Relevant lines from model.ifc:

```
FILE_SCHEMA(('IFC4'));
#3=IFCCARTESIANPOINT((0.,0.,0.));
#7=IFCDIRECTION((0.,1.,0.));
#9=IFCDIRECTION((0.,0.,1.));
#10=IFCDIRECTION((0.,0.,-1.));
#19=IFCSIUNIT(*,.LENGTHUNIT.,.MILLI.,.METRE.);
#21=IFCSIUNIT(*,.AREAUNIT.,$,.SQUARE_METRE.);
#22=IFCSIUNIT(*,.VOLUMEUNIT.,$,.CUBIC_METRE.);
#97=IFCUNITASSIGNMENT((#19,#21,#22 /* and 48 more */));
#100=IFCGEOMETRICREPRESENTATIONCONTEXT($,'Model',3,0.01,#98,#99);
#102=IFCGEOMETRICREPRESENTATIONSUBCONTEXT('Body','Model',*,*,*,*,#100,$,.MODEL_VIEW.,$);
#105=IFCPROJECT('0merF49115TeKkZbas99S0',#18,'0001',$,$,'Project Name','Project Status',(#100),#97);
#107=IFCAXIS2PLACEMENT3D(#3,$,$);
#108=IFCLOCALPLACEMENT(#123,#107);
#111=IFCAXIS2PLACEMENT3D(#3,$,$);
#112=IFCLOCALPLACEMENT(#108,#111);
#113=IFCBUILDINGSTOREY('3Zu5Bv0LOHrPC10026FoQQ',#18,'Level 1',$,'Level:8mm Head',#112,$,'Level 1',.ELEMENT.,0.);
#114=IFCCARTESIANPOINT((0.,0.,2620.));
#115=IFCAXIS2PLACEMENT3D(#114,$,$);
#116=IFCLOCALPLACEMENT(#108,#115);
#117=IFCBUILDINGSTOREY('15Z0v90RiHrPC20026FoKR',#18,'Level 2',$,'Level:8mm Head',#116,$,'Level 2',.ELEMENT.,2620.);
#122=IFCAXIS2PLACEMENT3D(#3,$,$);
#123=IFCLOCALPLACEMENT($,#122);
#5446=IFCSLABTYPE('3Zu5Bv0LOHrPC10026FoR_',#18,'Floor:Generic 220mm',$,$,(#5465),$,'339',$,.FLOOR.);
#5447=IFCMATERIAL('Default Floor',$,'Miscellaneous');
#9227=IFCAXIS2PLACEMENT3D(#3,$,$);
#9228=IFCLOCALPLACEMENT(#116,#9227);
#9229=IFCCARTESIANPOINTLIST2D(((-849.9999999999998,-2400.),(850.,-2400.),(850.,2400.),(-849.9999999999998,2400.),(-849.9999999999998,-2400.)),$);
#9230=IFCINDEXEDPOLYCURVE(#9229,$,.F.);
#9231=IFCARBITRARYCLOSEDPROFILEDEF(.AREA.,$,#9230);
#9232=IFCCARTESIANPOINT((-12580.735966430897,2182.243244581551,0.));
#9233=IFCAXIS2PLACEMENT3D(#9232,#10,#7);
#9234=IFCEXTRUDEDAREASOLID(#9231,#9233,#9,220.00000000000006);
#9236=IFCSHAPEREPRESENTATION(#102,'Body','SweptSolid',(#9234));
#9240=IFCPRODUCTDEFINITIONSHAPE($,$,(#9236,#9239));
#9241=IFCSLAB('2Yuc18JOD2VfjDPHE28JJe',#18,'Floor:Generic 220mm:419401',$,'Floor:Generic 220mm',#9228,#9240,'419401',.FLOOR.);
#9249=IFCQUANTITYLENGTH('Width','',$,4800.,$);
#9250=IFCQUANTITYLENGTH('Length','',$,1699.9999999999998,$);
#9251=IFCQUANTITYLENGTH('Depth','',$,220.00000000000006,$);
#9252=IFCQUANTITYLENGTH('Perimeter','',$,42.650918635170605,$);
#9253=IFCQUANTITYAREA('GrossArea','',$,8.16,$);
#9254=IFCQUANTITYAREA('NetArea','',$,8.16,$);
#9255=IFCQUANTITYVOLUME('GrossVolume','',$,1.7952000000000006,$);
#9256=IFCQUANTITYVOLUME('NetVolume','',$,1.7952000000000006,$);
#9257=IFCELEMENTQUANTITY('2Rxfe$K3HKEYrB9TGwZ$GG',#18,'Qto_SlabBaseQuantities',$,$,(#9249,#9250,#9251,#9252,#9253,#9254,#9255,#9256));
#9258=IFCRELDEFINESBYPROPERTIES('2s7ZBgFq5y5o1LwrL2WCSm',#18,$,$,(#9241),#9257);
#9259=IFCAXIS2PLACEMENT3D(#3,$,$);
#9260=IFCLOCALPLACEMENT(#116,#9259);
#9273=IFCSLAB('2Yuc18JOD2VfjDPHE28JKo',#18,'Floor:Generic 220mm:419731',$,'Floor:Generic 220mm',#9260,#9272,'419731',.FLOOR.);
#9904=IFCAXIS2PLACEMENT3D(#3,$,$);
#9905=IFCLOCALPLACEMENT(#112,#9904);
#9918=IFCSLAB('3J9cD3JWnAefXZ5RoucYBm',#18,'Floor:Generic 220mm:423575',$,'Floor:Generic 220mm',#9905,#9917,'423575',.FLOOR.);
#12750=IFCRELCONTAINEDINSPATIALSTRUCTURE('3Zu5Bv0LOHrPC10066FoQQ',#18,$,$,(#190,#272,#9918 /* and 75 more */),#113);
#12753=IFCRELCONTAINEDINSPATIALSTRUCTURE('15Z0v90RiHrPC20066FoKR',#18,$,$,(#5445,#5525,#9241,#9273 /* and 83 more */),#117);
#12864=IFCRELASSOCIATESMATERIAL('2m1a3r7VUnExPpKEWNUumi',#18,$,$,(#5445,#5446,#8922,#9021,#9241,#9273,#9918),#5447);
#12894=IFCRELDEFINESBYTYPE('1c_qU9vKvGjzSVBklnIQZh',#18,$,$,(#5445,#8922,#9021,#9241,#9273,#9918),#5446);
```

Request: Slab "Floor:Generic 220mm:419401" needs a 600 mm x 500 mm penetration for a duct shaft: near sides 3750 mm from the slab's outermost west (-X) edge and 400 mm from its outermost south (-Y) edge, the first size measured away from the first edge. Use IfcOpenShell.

```python
import numpy as np
import ifcopenshell
import ifcopenshell.api.feature
import ifcopenshell.api.geometry
import ifcopenshell.api.pset
import ifcopenshell.api.root
import ifcopenshell.geom
import ifcopenshell.util.element
import ifcopenshell.util.placement
import ifcopenshell.util.representation
import ifcopenshell.util.shape
import ifcopenshell.util.unit

model = ifcopenshell.open("model.ifc")
unit_scale = ifcopenshell.util.unit.calculate_unit_scale(model)
area_scale = ifcopenshell.util.unit.calculate_unit_scale(model, "AREAUNIT")
volume_scale = ifcopenshell.util.unit.calculate_unit_scale(model, "VOLUMEUNIT")
settings = ifcopenshell.geom.settings()


def volume(element):
    """Net volume in cubic metres, openings subtracted."""
    shape = ifcopenshell.geom.create_shape(settings, element)
    return ifcopenshell.util.shape.get_volume(shape.geometry)


slab = model.by_guid("2Yuc18JOD2VfjDPHE28JJe")
before = volume(slab)

# Extent in the slab's own axes, in metres. The edges named are its -X and -Y sides.
slab_shape = ifcopenshell.geom.create_shape(settings, slab)
vertices = ifcopenshell.util.shape.get_vertices(slab_shape.geometry)
x_min, y_min, bottom = vertices.min(axis=0)
top = vertices[:, 2].max()

opening = ifcopenshell.api.root.create_entity(model, ifc_class="IfcOpeningElement", name="Duct shaft opening", predefined_type="OPENING")
context = ifcopenshell.util.representation.get_context(model, "Model", "Body", "MODEL_VIEW")
width, depth = 0.6, 0.5
outline = [(0.0, 0.0), (width, 0.0), (width, depth), (0.0, depth), (0.0, 0.0)]
# Overshoot both faces by 50 mm so the cut is clean.
shape = ifcopenshell.api.geometry.add_slab_representation(
    model, context=context, depth=top - bottom + 0.1, polyline=outline
)
ifcopenshell.api.geometry.assign_representation(model, product=opening, representation=shape)

matrix = ifcopenshell.util.placement.get_local_placement(slab.ObjectPlacement)
matrix[:, 3] = matrix @ np.append(np.array([x_min + 3.75, y_min + 0.4, bottom - 0.05]) / unit_scale, 1.0)
ifcopenshell.api.geometry.edit_object_placement(model, product=opening, matrix=matrix, is_si=False)
ifcopenshell.api.feature.add_feature(model, feature=opening, element=slab)

after = volume(slab)

# Update the slab's stored quantities.
qto = model.by_id(ifcopenshell.util.element.get_pset(slab, "Qto_SlabBaseQuantities", should_inherit=False)["id"])
ifcopenshell.api.pset.edit_qto(model, qto=qto, properties={
    "NetArea": after / (top - bottom) / area_scale,
    "NetVolume": after / volume_scale,
})

print(f"slab volume {before:.3f} -> {after:.3f} m3")

model.write("model_updated.ifc")
```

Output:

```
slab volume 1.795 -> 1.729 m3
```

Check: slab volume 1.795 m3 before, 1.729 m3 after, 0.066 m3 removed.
